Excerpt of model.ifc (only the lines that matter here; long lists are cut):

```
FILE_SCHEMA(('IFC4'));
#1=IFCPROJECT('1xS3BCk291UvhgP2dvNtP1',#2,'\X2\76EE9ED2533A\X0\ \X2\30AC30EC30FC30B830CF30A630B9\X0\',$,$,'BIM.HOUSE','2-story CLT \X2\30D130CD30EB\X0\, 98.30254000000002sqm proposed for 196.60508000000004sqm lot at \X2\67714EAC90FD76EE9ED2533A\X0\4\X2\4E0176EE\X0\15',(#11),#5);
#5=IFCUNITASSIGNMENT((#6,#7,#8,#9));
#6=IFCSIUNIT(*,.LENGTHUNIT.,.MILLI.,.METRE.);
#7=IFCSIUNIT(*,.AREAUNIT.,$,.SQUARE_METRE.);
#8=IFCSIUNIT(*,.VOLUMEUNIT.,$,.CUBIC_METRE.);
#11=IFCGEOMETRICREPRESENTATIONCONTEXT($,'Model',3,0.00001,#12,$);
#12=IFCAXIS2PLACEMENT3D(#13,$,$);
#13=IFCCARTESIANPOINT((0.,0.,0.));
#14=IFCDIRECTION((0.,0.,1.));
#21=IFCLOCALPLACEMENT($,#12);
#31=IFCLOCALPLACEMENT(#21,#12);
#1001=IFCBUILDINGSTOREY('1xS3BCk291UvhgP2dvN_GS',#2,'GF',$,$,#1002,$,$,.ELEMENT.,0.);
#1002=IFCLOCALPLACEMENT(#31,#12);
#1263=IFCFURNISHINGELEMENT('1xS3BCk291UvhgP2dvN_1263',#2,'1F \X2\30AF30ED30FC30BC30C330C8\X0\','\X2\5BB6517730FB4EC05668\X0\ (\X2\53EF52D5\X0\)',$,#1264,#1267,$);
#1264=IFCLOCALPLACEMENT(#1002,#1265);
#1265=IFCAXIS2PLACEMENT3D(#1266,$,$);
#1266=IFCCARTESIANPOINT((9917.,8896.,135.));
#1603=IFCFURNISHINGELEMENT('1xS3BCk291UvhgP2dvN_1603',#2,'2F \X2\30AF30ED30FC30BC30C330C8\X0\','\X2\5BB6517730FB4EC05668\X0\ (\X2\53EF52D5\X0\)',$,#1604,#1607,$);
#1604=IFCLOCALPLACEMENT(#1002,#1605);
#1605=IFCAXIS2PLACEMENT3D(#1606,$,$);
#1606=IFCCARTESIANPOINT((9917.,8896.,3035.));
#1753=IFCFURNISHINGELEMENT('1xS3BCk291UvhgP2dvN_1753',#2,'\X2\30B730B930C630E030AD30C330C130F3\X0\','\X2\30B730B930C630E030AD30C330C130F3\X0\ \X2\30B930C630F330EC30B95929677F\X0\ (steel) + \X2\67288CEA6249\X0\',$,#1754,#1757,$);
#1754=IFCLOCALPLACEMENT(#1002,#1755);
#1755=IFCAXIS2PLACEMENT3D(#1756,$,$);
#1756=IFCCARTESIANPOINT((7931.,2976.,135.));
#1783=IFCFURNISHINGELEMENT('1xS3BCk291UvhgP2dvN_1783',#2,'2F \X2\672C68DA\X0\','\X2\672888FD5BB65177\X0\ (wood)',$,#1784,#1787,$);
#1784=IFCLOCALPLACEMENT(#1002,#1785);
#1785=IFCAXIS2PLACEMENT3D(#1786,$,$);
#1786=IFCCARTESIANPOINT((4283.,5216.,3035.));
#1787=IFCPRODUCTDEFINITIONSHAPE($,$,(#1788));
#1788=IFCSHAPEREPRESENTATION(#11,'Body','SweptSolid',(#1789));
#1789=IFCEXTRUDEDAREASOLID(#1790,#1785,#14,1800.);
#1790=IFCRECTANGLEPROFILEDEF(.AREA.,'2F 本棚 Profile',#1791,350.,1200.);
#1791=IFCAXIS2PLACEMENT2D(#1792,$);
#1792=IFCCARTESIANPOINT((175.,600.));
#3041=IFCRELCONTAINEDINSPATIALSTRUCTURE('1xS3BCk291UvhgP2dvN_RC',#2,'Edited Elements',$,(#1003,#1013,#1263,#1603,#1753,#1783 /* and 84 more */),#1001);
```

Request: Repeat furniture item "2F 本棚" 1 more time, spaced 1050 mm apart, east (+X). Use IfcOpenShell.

```python
import numpy as np
import ifcopenshell
import ifcopenshell.api.geometry
import ifcopenshell.api.root
import ifcopenshell.util.element
import ifcopenshell.util.placement
import ifcopenshell.util.unit

model = ifcopenshell.open("model.ifc")
unit_scale = ifcopenshell.util.unit.calculate_unit_scale(model)


def reuse_history(source, copy):
    """copy_class also copies each property set's owner history, people and application; keep the originals."""
    for rel in copy.IsDefinedBy:
        if rel.is_a("IfcRelDefinesByProperties") and (history := rel.RelatingPropertyDefinition.OwnerHistory):
            rel.RelatingPropertyDefinition.OwnerHistory = source.OwnerHistory
            ifcopenshell.util.element.remove_deep2(model, history)


source = model.by_guid("1xS3BCk291UvhgP2dvN_1783")
base = ifcopenshell.util.placement.get_local_placement(source.ObjectPlacement)
step = np.array([1.0, 0.0, 0.0]) * 1.05 / unit_scale

for i in range(1, 2):
    copy = ifcopenshell.api.root.copy_class(model, product=source)
    copy.Representation = ifcopenshell.util.element.copy_deep(
        model, source.Representation, exclude=["IfcGeometricRepresentationContext", "IfcRepresentationMap"]
    )
    reuse_history(source, copy)
    matrix = base.copy()
    matrix[:3, 3] += i * step
    print("added at", matrix[:3, 3].round(3) + 0.0)
    ifcopenshell.api.geometry.edit_object_placement(model, product=copy, matrix=matrix, is_si=False)

model.write("model-out.ifc")
```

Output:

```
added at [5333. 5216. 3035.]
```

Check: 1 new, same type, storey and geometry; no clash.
